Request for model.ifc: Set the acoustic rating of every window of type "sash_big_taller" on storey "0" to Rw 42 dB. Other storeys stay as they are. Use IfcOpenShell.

First a look at what the model holds.

```python
import ifcopenshell
import ifcopenshell.util.element

model = ifcopenshell.open("model.ifc")
print(model.schema)
storey = next(s for s in model.by_type("IfcBuildingStorey") if s.Name == "0")
windows = [e for e in ifcopenshell.util.element.get_decomposition(storey) if e.is_a("IfcWindow")]
seen = {}
for e in windows:
    element_type = ifcopenshell.util.element.get_type(e)
    key = (element_type.Name if element_type != e and element_type else None, ifcopenshell.util.element.get_pset(e, "Pset_WindowCommon", "AcousticRating"))
    seen[key] = seen.get(key, 0) + 1
for (name, value), count in sorted(seen.items(), key=str):
    print(count, "x", name, "|", value)
```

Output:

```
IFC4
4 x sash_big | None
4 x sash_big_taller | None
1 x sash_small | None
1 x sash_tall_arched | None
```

```python
import ifcopenshell
import ifcopenshell.api.pset
import ifcopenshell.util.element

model = ifcopenshell.open("model.ifc")

storey = next(s for s in model.by_type("IfcBuildingStorey") if s.Name == "0")
windows = [e for e in ifcopenshell.util.element.get_decomposition(storey) if e.is_a("IfcWindow")]

count = 0
for e in windows:
    element_type = ifcopenshell.util.element.get_type(e)
    if element_type in (None, e) or element_type.Name != "sash_big_taller":
        continue
    # add_pset returns the element's existing set when there is one.
    pset = ifcopenshell.api.pset.add_pset(model, product=e, name="Pset_WindowCommon")
    ifcopenshell.api.pset.edit_pset(model, pset=pset, properties={"AcousticRating": "Rw 42 dB"})
    count += 1

print(count, "windows updated")

model.write("model_v2.ifc")
```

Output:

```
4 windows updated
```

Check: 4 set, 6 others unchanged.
